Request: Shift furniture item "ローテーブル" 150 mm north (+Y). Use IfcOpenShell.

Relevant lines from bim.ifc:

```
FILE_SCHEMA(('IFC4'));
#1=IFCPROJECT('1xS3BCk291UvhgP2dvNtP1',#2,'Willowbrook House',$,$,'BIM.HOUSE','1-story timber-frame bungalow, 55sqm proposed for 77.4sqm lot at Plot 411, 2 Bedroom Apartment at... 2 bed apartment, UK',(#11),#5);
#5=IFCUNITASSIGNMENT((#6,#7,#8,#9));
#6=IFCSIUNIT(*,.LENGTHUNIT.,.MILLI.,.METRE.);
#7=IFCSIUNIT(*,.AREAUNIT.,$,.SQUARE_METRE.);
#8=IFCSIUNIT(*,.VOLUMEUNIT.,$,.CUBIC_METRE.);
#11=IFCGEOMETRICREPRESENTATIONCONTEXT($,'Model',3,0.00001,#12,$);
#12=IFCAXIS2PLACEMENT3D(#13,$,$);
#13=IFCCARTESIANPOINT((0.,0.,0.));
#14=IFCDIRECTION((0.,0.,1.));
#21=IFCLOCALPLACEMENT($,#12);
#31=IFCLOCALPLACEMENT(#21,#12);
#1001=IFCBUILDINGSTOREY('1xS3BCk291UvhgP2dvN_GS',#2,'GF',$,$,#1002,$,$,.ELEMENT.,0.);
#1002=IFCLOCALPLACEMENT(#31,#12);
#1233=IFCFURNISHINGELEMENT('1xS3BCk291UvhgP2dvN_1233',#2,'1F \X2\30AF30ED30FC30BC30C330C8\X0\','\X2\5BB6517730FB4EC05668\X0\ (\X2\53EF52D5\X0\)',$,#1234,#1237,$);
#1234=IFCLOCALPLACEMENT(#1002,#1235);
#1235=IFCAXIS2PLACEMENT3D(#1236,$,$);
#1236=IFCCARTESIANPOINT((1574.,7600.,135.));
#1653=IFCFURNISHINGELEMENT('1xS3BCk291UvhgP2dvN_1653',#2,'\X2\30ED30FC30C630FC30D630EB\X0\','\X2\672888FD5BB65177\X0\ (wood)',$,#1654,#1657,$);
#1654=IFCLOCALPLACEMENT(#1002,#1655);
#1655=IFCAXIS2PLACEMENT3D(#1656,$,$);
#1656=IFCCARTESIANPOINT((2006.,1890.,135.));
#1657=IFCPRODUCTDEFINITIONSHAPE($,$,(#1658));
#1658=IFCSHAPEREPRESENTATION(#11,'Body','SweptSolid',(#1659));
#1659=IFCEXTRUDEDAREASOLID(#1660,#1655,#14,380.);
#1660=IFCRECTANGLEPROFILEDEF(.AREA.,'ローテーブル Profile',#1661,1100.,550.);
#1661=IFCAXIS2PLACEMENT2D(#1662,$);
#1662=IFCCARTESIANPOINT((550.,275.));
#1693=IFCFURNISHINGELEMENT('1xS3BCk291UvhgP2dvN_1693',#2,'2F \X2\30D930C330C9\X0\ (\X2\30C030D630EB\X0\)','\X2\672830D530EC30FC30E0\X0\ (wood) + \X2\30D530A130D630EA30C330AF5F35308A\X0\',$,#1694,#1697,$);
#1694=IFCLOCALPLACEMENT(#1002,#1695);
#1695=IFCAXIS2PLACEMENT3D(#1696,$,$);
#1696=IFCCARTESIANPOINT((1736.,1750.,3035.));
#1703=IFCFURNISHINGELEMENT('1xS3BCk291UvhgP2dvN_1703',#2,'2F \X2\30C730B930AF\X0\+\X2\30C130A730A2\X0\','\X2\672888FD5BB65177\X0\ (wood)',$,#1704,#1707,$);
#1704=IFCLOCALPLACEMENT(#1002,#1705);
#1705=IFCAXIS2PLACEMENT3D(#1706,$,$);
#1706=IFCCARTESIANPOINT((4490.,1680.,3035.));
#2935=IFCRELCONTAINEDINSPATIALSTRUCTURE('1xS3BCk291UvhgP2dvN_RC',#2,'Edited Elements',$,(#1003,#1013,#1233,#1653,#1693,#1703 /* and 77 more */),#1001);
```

```python
import ifcopenshell
import ifcopenshell.api.geometry
import ifcopenshell.util.placement

model = ifcopenshell.open("bim.ifc")

item = model.by_guid("1xS3BCk291UvhgP2dvN_1653")
matrix = ifcopenshell.util.placement.get_local_placement(item.ObjectPlacement)
matrix[1, 3] += 150.0
ifcopenshell.api.geometry.edit_object_placement(model, product=item, matrix=matrix, is_si=False)

print(ifcopenshell.util.placement.get_local_placement(item.ObjectPlacement).round(3) + 0.0)

model.write("bim_updated.ifc")
```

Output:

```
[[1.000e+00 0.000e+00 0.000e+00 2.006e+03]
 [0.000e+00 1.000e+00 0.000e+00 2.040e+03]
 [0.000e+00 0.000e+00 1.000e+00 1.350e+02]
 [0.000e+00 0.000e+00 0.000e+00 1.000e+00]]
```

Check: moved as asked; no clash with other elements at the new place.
